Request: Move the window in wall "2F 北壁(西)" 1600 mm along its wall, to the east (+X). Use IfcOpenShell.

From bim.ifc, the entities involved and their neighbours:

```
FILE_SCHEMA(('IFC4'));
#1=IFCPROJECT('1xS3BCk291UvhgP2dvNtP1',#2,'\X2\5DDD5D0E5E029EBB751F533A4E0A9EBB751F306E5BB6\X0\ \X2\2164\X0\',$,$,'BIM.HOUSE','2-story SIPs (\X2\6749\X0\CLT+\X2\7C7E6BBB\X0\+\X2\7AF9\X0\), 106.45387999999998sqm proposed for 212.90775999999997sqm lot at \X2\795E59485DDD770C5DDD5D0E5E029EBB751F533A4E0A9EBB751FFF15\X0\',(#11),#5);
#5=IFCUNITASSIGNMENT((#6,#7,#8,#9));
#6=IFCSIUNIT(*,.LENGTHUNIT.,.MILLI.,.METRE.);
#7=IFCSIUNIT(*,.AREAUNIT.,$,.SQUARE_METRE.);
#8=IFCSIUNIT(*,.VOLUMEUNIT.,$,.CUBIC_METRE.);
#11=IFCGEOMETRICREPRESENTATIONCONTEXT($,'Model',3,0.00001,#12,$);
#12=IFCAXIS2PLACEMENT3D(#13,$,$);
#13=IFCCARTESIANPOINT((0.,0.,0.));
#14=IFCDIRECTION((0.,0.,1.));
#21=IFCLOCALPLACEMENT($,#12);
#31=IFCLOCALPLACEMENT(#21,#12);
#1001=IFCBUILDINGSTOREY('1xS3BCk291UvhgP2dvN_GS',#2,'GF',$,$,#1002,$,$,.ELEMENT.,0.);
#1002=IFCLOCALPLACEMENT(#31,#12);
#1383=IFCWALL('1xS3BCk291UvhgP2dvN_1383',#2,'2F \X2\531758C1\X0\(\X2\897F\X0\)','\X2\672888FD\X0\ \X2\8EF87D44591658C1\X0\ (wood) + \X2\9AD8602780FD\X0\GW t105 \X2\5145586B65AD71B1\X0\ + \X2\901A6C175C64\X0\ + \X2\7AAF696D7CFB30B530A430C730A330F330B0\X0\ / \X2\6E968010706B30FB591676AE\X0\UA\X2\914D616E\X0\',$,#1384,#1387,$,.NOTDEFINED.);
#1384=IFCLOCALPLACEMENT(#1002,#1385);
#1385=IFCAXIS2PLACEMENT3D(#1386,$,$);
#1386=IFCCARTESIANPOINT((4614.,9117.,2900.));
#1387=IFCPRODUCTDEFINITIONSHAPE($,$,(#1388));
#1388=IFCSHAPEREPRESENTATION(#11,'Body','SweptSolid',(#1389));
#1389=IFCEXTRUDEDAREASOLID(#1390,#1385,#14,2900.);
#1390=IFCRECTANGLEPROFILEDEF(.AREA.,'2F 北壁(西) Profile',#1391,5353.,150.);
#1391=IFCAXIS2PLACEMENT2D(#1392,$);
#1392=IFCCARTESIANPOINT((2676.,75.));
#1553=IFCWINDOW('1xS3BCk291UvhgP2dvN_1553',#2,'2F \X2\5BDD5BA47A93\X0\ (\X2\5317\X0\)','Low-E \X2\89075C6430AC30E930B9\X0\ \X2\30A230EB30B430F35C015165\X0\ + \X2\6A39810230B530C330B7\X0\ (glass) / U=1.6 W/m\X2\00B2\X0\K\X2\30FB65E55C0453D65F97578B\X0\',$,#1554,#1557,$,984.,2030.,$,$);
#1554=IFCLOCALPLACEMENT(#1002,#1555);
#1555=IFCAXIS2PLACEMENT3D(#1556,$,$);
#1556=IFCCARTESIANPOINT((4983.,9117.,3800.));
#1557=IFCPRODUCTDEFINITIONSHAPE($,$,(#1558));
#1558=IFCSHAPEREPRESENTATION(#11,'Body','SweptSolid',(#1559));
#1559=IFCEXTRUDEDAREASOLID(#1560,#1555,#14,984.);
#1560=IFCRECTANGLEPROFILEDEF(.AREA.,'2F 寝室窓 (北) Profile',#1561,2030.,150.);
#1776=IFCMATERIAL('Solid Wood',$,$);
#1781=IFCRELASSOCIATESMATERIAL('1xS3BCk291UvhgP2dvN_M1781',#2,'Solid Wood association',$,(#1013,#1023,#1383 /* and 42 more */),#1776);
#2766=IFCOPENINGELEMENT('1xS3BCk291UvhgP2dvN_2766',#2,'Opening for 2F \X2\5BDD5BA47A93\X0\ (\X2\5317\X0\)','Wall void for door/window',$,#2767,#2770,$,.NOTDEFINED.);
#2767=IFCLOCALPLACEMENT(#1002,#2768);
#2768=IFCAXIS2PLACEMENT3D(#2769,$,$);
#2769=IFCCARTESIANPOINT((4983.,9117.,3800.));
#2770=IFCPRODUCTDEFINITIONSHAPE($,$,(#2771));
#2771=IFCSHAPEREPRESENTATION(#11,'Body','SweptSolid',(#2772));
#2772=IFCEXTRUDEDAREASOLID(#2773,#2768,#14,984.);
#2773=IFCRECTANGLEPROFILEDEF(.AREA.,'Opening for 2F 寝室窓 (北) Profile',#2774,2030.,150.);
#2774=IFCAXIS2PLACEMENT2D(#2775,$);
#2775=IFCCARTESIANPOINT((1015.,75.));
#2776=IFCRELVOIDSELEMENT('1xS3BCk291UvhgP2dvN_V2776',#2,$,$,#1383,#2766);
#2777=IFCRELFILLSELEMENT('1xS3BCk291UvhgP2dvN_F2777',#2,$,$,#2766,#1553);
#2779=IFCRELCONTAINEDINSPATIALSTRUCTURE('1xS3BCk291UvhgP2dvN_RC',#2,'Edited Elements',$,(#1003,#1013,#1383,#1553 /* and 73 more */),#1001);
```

```python
import ifcopenshell
import ifcopenshell.api.geometry
import ifcopenshell.util.placement
import ifcopenshell.util.unit

model = ifcopenshell.open("bim.ifc")
unit_scale = ifcopenshell.util.unit.calculate_unit_scale(model)

window = model.by_guid("1xS3BCk291UvhgP2dvN_1553")
opening = window.FillsVoids[0].RelatingOpeningElement
wall = opening.VoidsElements[0].RelatingBuildingElement

wall_matrix = ifcopenshell.util.placement.get_local_placement(wall.ObjectPlacement)
shift = wall_matrix[:3, 0] * 1.6 / unit_scale
before = ifcopenshell.util.placement.get_local_placement(window.ObjectPlacement)[:3, 3].copy()

# The window is not placed relative to its opening, so move both.
for product in (opening, window):
    matrix = ifcopenshell.util.placement.get_local_placement(product.ObjectPlacement)
    matrix[:3, 3] += shift
    ifcopenshell.api.geometry.edit_object_placement(model, product=product, matrix=matrix, is_si=False)

after = ifcopenshell.util.placement.get_local_placement(window.ObjectPlacement)[:3, 3]
print("window moved by", (after - before).round(3) + 0.0)

model.write("bim_edited.ifc")
```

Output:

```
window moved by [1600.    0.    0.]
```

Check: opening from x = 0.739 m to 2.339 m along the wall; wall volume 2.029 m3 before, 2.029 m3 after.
